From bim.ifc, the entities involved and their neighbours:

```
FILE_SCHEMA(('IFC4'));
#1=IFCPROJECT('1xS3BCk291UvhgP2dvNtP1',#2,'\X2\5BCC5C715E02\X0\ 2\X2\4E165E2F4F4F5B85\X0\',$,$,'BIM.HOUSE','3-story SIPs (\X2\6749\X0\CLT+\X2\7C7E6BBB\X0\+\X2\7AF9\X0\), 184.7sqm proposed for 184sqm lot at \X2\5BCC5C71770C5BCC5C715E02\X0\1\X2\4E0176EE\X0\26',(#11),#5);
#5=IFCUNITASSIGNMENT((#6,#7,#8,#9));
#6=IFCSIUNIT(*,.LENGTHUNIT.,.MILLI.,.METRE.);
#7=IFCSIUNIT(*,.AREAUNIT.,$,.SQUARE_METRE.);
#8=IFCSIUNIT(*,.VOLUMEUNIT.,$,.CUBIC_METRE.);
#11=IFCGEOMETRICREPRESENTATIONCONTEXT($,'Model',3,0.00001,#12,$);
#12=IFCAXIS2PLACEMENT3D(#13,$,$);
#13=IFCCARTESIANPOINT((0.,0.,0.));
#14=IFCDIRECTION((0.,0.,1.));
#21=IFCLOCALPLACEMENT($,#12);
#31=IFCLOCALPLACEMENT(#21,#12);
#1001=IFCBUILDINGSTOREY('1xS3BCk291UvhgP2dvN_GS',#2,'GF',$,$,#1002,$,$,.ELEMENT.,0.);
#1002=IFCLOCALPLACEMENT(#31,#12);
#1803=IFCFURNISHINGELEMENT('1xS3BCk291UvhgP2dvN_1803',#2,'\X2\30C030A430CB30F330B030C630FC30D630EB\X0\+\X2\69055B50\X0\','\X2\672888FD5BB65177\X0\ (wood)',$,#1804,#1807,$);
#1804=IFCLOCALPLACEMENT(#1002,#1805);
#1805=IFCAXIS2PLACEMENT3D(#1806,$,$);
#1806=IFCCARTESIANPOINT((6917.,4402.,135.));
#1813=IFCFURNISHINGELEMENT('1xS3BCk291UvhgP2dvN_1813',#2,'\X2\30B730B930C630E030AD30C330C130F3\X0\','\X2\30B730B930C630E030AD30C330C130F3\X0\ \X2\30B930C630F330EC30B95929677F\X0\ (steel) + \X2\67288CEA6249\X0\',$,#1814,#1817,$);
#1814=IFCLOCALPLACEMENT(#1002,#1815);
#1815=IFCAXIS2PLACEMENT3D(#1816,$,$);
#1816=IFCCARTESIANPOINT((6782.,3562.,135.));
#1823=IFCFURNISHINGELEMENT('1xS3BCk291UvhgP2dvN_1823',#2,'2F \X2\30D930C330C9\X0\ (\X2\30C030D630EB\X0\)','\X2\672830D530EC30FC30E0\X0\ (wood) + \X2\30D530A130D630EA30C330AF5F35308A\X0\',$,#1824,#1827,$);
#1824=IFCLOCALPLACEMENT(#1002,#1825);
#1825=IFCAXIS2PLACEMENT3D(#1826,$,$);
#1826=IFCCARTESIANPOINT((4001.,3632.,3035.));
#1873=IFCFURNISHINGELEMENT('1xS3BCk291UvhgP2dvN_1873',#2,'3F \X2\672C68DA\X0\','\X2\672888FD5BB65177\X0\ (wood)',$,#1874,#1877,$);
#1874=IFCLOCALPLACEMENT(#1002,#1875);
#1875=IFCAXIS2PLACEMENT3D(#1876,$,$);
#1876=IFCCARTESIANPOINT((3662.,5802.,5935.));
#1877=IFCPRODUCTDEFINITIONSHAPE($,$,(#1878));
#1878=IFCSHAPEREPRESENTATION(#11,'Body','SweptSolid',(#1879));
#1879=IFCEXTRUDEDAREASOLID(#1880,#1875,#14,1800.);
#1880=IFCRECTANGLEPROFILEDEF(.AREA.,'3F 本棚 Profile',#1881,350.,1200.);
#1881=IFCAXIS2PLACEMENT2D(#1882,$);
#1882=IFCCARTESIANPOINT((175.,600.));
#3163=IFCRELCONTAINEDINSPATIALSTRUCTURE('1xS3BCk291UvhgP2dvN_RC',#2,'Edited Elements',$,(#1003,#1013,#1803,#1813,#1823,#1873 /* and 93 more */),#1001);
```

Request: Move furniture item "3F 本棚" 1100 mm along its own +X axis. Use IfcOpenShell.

```python
import ifcopenshell
import ifcopenshell.api.geometry
import ifcopenshell.util.placement
import ifcopenshell.util.unit

model = ifcopenshell.open("bim.ifc")
unit_scale = ifcopenshell.util.unit.calculate_unit_scale(model)

item = model.by_id(1873)
matrix = ifcopenshell.util.placement.get_local_placement(item.ObjectPlacement)
matrix[:3, 3] += matrix[:3, 0] * 1.1 / unit_scale
ifcopenshell.api.geometry.edit_object_placement(model, product=item, matrix=matrix, is_si=False)

print(ifcopenshell.util.placement.get_local_placement(item.ObjectPlacement).round(3) + 0.0)

model.write("bim_rev.ifc")
```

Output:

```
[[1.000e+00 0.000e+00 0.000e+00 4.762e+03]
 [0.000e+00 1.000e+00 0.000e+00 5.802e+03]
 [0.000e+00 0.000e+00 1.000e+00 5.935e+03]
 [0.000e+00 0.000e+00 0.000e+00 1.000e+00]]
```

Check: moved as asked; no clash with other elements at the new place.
